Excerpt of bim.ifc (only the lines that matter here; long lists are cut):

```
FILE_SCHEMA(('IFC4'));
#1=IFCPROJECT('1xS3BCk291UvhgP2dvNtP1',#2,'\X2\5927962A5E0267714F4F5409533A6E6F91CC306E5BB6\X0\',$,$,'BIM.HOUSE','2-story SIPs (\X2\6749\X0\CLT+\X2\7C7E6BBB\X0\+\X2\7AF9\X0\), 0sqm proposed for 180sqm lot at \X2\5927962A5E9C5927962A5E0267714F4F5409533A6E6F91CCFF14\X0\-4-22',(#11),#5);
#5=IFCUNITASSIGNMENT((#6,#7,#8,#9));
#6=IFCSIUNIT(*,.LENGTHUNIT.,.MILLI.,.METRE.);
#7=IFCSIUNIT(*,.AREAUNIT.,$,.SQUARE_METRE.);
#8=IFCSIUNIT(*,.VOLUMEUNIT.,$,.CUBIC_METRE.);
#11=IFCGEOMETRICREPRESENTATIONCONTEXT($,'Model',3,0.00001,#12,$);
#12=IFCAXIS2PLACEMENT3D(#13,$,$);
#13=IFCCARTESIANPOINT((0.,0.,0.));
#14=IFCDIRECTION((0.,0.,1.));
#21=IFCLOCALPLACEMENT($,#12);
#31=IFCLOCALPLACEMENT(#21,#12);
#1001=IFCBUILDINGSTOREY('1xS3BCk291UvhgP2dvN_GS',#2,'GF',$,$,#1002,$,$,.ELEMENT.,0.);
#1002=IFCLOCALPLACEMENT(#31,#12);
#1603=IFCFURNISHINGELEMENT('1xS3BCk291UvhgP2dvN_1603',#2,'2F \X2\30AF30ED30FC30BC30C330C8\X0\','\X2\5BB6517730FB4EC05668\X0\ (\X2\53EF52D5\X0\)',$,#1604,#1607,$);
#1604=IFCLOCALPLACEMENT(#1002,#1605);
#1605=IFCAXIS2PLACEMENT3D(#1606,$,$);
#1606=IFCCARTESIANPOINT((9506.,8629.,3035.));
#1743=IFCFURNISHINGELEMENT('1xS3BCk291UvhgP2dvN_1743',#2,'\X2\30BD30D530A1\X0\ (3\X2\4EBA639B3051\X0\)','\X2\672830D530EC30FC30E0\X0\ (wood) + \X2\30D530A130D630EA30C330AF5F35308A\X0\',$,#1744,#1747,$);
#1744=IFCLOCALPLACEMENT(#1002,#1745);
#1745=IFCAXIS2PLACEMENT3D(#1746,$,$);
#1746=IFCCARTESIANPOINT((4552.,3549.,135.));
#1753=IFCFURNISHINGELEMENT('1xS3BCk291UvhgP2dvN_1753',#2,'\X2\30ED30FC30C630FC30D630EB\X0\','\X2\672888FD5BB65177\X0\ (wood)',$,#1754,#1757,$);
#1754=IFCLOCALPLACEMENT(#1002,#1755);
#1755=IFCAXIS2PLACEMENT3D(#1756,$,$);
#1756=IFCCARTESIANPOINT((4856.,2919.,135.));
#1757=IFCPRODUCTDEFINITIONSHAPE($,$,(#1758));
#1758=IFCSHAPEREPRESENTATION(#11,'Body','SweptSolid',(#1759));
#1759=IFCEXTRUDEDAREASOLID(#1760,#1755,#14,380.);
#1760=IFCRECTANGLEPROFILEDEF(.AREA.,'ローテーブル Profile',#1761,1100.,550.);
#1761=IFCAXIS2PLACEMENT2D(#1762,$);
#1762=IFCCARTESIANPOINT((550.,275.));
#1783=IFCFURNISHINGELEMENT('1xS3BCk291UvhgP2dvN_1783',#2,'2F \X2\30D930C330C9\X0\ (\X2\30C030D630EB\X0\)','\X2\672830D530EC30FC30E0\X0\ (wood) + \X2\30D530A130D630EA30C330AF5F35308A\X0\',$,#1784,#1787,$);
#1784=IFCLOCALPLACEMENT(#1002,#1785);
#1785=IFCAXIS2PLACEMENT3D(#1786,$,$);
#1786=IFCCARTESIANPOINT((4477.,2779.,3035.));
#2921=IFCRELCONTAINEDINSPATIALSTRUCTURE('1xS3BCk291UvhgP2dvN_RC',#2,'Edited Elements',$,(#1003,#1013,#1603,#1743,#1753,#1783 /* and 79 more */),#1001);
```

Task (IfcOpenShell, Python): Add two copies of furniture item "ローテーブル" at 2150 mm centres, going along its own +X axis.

```python
import ifcopenshell
import ifcopenshell.api.geometry
import ifcopenshell.api.root
import ifcopenshell.util.element
import ifcopenshell.util.placement
import ifcopenshell.util.unit

model = ifcopenshell.open("bim.ifc")
unit_scale = ifcopenshell.util.unit.calculate_unit_scale(model)


def reuse_history(source, copy):
    """copy_class also copies each property set's owner history, people and application; keep the originals."""
    for rel in copy.IsDefinedBy:
        if rel.is_a("IfcRelDefinesByProperties") and (history := rel.RelatingPropertyDefinition.OwnerHistory):
            rel.RelatingPropertyDefinition.OwnerHistory = source.OwnerHistory
            ifcopenshell.util.element.remove_deep2(model, history)


source = model.by_guid("1xS3BCk291UvhgP2dvN_1753")
base = ifcopenshell.util.placement.get_local_placement(source.ObjectPlacement)
step = base[:3, 0] * 2.15 / unit_scale

for i in range(1, 3):
    copy = ifcopenshell.api.root.copy_class(model, product=source)
    copy.Representation = ifcopenshell.util.element.copy_deep(
        model, source.Representation, exclude=["IfcGeometricRepresentationContext", "IfcRepresentationMap"]
    )
    reuse_history(source, copy)
    matrix = base.copy()
    matrix[:3, 3] += i * step
    print("added at", matrix[:3, 3].round(3) + 0.0)
    ifcopenshell.api.geometry.edit_object_placement(model, product=copy, matrix=matrix, is_si=False)

model.write("bim_v2.ifc")
```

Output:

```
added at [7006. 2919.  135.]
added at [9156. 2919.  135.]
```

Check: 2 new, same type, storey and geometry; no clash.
